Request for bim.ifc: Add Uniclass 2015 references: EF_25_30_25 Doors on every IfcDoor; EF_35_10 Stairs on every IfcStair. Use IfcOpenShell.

First a look at what the model holds.

```python
import ifcopenshell

model = ifcopenshell.open("bim.ifc")
print(model.schema)
print("classifications:", [c.Name for c in model.by_type("IfcClassification")])
for ifc_class in ("IfcDoor", "IfcRoof", "IfcStair", "IfcWall", "IfcWindow"):
    print(ifc_class, len(model.by_type(ifc_class)))
```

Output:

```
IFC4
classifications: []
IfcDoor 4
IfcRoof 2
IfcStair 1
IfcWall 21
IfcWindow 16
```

```python
import ifcopenshell
import ifcopenshell.api.classification

model = ifcopenshell.open("bim.ifc")

system = ifcopenshell.api.classification.add_classification(model, classification="Uniclass 2015")

codes = {
    "IfcDoor": ("EF_25_30_25", "Doors"),
    "IfcStair": ("EF_35_10", "Stairs"),
}
for ifc_class, (code, name) in codes.items():
    products = model.by_type(ifc_class)
    ifcopenshell.api.classification.add_reference(
        model, products=products, classification=system, identification=code, name=name
    )
    print(code, len(products))

model.write("bim_updated.ifc")
```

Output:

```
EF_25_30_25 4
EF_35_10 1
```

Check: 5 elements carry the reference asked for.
